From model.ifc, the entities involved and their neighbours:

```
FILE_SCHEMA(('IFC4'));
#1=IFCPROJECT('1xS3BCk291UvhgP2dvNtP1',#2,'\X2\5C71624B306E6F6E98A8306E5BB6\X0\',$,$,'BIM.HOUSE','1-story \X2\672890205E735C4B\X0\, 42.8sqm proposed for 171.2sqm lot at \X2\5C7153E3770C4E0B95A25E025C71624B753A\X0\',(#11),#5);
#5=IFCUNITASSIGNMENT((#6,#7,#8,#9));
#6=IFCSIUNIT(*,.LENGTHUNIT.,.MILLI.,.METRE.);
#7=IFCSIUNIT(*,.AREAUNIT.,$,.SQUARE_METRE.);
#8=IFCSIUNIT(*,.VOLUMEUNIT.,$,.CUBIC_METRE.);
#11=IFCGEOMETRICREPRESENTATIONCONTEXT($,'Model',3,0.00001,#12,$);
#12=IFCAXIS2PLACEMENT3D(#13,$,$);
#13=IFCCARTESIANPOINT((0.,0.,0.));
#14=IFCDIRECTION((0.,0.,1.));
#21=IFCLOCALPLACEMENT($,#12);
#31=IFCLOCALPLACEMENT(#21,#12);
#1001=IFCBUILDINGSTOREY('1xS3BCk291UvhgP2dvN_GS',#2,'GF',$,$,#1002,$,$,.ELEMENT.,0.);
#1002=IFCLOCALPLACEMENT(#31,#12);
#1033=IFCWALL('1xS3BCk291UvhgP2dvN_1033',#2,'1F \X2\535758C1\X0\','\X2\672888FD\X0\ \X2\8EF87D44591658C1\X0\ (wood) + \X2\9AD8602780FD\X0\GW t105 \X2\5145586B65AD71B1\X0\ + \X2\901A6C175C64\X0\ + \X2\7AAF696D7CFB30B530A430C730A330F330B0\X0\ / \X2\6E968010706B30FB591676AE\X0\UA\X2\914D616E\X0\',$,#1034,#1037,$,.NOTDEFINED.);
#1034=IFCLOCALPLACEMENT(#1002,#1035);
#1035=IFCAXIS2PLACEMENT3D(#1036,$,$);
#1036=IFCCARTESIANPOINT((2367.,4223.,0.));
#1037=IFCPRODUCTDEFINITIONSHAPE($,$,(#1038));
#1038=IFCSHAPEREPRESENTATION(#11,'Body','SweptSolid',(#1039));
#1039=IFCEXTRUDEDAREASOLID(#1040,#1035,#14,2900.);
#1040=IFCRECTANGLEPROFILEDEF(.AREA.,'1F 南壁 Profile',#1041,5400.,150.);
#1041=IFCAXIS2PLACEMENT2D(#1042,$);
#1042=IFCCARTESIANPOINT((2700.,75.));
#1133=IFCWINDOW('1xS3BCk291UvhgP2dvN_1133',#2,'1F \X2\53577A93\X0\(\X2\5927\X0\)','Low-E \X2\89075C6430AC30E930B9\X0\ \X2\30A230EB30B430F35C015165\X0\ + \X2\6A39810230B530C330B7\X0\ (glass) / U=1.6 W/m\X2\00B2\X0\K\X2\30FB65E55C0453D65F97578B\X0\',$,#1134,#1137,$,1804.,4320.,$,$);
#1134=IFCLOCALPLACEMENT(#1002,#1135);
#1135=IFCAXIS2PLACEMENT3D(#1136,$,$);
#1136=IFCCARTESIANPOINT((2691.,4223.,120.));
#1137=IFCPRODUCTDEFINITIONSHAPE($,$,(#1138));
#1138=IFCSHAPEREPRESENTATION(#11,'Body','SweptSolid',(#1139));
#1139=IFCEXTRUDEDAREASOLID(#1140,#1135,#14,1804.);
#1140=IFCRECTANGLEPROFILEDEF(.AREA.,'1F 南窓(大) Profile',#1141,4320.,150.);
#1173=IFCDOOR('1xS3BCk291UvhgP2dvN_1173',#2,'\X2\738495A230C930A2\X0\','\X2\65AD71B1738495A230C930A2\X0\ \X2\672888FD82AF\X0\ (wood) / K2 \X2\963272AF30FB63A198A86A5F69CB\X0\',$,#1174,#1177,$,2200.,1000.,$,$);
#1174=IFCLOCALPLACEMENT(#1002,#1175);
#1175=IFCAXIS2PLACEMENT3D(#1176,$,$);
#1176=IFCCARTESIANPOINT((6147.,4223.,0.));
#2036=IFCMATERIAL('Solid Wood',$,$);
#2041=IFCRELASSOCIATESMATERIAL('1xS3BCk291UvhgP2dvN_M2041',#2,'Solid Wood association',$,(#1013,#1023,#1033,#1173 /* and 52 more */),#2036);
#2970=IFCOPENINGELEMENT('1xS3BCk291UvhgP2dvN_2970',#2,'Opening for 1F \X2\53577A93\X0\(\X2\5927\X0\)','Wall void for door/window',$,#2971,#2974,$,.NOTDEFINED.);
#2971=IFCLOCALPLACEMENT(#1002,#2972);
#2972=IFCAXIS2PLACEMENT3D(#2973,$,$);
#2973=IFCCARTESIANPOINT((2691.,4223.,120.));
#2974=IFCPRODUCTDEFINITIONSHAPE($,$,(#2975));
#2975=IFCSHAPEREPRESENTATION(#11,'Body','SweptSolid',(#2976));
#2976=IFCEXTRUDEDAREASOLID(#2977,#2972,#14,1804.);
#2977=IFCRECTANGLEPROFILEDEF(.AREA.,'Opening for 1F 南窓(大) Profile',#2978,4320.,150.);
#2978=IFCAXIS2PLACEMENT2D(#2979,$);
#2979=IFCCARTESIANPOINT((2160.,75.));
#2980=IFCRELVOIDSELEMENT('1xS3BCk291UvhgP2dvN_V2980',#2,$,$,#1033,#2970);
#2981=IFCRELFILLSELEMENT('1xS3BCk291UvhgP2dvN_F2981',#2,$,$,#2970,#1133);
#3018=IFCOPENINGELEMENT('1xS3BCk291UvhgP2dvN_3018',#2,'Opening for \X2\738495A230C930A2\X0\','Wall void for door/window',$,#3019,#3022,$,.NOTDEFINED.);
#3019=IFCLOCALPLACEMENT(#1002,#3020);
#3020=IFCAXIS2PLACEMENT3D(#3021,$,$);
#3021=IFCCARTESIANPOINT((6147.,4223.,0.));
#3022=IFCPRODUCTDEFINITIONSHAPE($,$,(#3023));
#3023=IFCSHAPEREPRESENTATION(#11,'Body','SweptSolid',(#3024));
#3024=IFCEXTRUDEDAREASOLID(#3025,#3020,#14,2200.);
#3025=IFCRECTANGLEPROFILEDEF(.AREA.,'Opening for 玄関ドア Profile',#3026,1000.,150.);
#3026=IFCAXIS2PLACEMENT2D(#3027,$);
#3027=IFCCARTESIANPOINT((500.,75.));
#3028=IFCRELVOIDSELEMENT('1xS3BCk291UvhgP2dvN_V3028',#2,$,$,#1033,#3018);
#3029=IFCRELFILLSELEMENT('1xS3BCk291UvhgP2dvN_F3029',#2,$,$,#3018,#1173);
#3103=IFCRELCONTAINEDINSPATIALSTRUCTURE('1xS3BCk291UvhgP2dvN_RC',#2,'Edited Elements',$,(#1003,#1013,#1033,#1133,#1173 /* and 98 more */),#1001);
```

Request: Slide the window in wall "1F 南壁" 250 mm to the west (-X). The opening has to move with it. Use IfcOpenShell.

```python
import ifcopenshell
import ifcopenshell.api.geometry
import ifcopenshell.util.placement
import ifcopenshell.util.unit

model = ifcopenshell.open("model.ifc")
unit_scale = ifcopenshell.util.unit.calculate_unit_scale(model)

window = model.by_id(1133)
opening = window.FillsVoids[0].RelatingOpeningElement
wall = opening.VoidsElements[0].RelatingBuildingElement

wall_matrix = ifcopenshell.util.placement.get_local_placement(wall.ObjectPlacement)
shift = wall_matrix[:3, 0] * -0.25 / unit_scale
before = ifcopenshell.util.placement.get_local_placement(window.ObjectPlacement)[:3, 3].copy()

# The window is not placed relative to its opening, so move both.
for product in (opening, window):
    matrix = ifcopenshell.util.placement.get_local_placement(product.ObjectPlacement)
    matrix[:3, 3] += shift
    ifcopenshell.api.geometry.edit_object_placement(model, product=product, matrix=matrix, is_si=False)

after = ifcopenshell.util.placement.get_local_placement(window.ObjectPlacement)[:3, 3]
print("window moved by", (after - before).round(3) + 0.0)

model.write("model_updated.ifc")
```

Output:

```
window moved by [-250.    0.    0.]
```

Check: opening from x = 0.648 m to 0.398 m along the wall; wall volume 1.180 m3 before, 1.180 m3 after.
